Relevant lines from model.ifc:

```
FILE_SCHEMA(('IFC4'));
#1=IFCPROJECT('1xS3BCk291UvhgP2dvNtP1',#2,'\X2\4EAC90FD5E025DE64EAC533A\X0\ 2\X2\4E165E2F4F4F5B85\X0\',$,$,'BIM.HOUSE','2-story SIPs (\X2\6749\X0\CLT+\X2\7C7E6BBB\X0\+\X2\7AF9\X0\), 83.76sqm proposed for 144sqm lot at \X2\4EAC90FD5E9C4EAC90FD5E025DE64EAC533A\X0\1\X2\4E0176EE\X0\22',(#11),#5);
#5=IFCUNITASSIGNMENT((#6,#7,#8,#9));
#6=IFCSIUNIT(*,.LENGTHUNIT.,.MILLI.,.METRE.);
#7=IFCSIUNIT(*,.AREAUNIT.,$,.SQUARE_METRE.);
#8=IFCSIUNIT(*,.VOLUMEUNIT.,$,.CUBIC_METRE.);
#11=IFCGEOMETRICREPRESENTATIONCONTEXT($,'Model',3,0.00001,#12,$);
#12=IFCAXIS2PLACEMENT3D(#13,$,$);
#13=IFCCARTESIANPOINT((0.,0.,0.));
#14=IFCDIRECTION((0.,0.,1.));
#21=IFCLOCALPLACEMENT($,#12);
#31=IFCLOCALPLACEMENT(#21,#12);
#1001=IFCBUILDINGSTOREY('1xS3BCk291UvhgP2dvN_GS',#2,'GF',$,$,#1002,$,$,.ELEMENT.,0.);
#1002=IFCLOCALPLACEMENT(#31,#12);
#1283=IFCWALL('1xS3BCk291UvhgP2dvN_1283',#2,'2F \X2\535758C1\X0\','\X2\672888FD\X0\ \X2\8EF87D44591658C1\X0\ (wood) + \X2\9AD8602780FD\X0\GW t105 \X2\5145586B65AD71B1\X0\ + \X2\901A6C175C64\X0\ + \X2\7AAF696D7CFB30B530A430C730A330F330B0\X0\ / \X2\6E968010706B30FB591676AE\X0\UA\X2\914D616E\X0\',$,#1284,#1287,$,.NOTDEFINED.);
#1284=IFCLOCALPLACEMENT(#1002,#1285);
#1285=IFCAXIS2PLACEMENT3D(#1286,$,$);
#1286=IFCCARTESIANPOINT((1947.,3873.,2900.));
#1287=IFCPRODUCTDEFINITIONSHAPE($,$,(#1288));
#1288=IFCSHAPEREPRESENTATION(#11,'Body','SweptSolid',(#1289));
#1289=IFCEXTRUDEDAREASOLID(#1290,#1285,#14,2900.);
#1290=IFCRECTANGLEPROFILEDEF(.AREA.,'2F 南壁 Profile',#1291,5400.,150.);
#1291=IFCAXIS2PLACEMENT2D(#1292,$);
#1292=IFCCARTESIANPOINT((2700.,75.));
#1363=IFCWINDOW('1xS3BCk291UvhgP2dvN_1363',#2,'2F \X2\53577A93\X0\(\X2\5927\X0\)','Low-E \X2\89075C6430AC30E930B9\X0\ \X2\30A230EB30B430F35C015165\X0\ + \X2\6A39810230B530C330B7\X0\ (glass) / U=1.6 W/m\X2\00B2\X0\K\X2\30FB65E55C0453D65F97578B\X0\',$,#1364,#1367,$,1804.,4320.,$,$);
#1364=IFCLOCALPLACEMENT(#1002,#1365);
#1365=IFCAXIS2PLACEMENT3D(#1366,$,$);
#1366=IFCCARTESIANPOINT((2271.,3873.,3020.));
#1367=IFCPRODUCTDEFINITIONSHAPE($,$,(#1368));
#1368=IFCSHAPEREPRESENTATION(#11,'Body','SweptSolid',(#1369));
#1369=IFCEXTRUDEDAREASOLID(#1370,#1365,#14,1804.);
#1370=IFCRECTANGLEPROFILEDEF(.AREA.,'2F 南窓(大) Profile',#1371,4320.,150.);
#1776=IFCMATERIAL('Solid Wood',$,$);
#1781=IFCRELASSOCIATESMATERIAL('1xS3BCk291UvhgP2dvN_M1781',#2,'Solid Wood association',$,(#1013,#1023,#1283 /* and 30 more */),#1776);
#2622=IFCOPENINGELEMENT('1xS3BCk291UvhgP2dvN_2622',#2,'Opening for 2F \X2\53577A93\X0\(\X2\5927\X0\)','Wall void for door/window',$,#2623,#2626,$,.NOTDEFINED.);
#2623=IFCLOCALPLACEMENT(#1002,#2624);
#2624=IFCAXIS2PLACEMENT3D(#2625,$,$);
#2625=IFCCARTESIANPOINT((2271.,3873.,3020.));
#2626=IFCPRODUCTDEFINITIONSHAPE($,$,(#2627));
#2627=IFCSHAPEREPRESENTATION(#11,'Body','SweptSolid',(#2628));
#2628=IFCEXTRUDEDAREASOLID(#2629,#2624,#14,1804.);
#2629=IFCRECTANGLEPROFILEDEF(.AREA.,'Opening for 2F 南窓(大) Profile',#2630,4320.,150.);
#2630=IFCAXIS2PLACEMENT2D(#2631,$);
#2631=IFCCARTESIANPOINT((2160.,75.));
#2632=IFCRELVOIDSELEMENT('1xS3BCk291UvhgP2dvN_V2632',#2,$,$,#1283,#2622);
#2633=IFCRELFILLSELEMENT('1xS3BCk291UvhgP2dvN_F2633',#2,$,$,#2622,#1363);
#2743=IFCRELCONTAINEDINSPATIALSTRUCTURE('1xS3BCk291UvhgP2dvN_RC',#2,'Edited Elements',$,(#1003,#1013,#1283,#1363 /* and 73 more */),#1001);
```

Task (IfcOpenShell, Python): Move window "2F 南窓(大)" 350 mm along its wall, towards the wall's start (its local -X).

```python
import ifcopenshell
import ifcopenshell.api.geometry
import ifcopenshell.util.placement

model = ifcopenshell.open("model.ifc")

window = model.by_id(1363)
opening = window.FillsVoids[0].RelatingOpeningElement
wall = opening.VoidsElements[0].RelatingBuildingElement

wall_matrix = ifcopenshell.util.placement.get_local_placement(wall.ObjectPlacement)
shift = wall_matrix[:3, 0] * -350.0
before = ifcopenshell.util.placement.get_local_placement(window.ObjectPlacement)[:3, 3].copy()

# The window is not placed relative to its opening, so move both.
for product in (opening, window):
    matrix = ifcopenshell.util.placement.get_local_placement(product.ObjectPlacement)
    matrix[:3, 3] += shift
    ifcopenshell.api.geometry.edit_object_placement(model, product=product, matrix=matrix, is_si=False)

after = ifcopenshell.util.placement.get_local_placement(window.ObjectPlacement)[:3, 3]
print("window moved by", (after - before).round(3) + 0.0)

model.write("model_v2.ifc")
```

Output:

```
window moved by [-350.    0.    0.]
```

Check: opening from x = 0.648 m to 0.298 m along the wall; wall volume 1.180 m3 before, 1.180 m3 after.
